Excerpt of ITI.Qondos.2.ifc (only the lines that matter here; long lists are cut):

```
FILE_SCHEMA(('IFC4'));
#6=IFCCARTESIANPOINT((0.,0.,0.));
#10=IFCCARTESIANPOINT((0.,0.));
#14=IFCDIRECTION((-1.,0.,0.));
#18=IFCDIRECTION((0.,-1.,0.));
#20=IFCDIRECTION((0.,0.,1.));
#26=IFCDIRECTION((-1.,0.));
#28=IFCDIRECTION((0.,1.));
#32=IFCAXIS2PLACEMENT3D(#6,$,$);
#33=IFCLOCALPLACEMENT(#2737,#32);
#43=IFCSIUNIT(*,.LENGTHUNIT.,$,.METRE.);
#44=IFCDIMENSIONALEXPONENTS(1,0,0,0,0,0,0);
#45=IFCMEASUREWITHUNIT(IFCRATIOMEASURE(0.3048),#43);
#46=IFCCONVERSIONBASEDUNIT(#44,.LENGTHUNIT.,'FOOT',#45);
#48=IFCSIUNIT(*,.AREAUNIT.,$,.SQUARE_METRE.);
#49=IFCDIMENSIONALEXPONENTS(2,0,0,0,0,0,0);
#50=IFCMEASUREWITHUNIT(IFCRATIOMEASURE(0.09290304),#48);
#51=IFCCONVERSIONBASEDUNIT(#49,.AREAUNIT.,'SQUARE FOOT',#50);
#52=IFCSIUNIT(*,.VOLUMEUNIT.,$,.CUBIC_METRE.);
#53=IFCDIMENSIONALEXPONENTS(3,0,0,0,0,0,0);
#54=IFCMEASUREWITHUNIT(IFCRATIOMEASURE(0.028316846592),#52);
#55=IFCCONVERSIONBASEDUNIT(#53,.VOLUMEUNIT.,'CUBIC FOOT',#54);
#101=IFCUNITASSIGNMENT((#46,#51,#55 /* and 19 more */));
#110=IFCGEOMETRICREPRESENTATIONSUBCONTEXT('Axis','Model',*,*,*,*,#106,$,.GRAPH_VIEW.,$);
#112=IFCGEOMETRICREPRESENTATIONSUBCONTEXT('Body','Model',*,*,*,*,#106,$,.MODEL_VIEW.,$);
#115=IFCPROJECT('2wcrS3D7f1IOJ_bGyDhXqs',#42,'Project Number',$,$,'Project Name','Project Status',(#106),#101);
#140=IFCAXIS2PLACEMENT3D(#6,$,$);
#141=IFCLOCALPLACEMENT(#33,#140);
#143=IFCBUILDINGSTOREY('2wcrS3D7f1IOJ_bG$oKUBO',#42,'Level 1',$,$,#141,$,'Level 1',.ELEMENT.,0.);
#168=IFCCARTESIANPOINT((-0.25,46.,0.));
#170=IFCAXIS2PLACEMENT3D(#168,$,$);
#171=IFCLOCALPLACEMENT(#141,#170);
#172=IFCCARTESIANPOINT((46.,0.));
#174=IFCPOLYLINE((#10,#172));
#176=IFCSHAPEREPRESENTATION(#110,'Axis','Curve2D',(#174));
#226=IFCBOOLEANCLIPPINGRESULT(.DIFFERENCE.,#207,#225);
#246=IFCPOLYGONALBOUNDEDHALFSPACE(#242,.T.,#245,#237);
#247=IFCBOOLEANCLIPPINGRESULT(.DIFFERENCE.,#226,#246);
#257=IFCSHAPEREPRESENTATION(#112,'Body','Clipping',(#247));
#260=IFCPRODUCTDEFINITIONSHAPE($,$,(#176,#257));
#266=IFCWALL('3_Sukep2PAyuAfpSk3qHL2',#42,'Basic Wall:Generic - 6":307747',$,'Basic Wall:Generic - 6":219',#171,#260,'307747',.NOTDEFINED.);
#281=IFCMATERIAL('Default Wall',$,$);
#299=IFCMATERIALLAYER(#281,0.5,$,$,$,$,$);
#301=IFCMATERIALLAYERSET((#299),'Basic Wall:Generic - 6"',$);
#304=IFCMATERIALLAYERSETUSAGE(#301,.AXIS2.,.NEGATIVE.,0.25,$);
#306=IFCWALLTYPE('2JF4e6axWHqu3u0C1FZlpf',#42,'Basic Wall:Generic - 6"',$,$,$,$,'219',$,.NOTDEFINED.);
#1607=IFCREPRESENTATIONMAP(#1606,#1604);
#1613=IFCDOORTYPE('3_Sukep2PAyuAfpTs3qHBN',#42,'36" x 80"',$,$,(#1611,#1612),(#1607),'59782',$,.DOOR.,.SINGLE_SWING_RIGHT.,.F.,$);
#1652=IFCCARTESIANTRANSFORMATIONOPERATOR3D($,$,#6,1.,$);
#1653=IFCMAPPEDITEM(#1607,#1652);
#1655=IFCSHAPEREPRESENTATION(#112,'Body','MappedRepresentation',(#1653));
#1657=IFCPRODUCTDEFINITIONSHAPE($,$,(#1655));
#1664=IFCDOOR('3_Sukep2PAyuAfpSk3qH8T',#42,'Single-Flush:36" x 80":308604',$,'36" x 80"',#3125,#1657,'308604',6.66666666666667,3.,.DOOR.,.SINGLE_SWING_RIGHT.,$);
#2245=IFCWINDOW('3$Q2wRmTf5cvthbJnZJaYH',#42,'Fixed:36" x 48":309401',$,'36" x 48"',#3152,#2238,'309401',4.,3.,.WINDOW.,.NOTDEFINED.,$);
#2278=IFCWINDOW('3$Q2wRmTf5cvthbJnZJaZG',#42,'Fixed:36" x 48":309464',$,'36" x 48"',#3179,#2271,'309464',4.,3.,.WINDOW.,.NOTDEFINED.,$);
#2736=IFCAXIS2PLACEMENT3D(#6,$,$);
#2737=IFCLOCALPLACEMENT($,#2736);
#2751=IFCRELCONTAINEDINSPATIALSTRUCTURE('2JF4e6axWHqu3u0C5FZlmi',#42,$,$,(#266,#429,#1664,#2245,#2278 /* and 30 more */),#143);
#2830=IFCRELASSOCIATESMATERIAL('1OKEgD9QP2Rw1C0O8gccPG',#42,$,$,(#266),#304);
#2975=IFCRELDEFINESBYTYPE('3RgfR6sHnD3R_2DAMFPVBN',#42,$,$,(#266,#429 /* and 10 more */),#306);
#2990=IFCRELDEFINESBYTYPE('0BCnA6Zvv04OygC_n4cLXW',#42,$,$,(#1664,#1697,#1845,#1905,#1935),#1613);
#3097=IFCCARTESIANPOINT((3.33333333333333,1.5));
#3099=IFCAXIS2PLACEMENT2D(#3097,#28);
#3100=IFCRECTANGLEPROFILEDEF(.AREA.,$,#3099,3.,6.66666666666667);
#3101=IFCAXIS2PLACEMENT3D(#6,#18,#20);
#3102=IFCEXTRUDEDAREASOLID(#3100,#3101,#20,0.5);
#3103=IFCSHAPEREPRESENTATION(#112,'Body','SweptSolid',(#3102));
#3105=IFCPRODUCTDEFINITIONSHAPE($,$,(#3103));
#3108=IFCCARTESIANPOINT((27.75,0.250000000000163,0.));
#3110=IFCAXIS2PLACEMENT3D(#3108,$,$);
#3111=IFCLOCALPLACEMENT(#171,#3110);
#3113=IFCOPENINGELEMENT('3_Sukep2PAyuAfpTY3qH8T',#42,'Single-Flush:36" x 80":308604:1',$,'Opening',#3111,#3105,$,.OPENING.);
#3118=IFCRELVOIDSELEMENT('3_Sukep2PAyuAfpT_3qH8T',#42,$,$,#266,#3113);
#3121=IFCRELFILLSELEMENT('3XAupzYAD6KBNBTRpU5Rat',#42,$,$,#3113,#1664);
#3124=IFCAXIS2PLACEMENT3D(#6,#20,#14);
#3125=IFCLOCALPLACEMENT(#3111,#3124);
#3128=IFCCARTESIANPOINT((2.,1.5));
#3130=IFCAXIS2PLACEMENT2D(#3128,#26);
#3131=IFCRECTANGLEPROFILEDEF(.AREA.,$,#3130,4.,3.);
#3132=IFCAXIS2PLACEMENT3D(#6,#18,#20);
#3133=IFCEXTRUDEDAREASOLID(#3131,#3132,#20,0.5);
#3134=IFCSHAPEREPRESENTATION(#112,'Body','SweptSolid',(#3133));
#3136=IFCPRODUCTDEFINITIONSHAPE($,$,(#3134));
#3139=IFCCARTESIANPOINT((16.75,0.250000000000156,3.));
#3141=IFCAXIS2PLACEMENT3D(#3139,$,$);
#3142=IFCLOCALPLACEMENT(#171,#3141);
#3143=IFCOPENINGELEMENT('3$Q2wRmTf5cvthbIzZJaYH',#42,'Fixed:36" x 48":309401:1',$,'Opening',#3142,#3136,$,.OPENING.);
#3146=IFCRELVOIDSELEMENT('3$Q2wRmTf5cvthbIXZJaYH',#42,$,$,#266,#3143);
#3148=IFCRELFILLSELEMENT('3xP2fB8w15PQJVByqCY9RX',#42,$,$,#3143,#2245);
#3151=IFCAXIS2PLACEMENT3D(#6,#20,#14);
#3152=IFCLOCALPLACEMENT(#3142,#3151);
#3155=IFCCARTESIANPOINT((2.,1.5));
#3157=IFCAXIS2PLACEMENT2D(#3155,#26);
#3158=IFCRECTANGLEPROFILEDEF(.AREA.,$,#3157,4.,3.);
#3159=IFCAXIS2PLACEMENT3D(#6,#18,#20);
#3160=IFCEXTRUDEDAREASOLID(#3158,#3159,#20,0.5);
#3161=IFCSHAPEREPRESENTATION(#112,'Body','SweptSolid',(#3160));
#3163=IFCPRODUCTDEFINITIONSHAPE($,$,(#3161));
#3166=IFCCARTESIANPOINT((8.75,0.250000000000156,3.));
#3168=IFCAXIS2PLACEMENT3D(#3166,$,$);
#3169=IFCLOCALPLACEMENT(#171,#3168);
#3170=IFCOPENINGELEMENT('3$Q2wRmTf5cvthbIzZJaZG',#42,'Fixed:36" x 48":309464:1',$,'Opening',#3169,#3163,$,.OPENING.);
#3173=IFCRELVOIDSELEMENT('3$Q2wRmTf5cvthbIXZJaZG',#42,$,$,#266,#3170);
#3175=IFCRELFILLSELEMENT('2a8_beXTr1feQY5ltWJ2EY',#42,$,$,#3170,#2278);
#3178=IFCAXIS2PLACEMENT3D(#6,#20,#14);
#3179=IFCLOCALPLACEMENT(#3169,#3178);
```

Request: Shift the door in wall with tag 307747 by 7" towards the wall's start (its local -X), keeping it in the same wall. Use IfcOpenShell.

```python
import ifcopenshell
import ifcopenshell.api.geometry
import ifcopenshell.util.placement
import ifcopenshell.util.unit

model = ifcopenshell.open("ITI.Qondos.2.ifc")
unit_scale = ifcopenshell.util.unit.calculate_unit_scale(model)

door = model.by_id(1664)
opening = door.FillsVoids[0].RelatingOpeningElement
wall = opening.VoidsElements[0].RelatingBuildingElement

wall_matrix = ifcopenshell.util.placement.get_local_placement(wall.ObjectPlacement)
shift = wall_matrix[:3, 0] * -7 * 0.0254 / unit_scale
before = ifcopenshell.util.placement.get_local_placement(door.ObjectPlacement)[:3, 3].copy()

# The door is placed relative to its opening, so it follows when the opening moves.
matrix = ifcopenshell.util.placement.get_local_placement(opening.ObjectPlacement)
matrix[:3, 3] += shift
ifcopenshell.api.geometry.edit_object_placement(
    model, product=opening, matrix=matrix, is_si=False, should_transform_children=True
)

after = ifcopenshell.util.placement.get_local_placement(door.ObjectPlacement)[:3, 3]
print("door moved by", (after - before).round(3) + 0.0)

model.write("ITI.Qondos.2_v2.ifc")
```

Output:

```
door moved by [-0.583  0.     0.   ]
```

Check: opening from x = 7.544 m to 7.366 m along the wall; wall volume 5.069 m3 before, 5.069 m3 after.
